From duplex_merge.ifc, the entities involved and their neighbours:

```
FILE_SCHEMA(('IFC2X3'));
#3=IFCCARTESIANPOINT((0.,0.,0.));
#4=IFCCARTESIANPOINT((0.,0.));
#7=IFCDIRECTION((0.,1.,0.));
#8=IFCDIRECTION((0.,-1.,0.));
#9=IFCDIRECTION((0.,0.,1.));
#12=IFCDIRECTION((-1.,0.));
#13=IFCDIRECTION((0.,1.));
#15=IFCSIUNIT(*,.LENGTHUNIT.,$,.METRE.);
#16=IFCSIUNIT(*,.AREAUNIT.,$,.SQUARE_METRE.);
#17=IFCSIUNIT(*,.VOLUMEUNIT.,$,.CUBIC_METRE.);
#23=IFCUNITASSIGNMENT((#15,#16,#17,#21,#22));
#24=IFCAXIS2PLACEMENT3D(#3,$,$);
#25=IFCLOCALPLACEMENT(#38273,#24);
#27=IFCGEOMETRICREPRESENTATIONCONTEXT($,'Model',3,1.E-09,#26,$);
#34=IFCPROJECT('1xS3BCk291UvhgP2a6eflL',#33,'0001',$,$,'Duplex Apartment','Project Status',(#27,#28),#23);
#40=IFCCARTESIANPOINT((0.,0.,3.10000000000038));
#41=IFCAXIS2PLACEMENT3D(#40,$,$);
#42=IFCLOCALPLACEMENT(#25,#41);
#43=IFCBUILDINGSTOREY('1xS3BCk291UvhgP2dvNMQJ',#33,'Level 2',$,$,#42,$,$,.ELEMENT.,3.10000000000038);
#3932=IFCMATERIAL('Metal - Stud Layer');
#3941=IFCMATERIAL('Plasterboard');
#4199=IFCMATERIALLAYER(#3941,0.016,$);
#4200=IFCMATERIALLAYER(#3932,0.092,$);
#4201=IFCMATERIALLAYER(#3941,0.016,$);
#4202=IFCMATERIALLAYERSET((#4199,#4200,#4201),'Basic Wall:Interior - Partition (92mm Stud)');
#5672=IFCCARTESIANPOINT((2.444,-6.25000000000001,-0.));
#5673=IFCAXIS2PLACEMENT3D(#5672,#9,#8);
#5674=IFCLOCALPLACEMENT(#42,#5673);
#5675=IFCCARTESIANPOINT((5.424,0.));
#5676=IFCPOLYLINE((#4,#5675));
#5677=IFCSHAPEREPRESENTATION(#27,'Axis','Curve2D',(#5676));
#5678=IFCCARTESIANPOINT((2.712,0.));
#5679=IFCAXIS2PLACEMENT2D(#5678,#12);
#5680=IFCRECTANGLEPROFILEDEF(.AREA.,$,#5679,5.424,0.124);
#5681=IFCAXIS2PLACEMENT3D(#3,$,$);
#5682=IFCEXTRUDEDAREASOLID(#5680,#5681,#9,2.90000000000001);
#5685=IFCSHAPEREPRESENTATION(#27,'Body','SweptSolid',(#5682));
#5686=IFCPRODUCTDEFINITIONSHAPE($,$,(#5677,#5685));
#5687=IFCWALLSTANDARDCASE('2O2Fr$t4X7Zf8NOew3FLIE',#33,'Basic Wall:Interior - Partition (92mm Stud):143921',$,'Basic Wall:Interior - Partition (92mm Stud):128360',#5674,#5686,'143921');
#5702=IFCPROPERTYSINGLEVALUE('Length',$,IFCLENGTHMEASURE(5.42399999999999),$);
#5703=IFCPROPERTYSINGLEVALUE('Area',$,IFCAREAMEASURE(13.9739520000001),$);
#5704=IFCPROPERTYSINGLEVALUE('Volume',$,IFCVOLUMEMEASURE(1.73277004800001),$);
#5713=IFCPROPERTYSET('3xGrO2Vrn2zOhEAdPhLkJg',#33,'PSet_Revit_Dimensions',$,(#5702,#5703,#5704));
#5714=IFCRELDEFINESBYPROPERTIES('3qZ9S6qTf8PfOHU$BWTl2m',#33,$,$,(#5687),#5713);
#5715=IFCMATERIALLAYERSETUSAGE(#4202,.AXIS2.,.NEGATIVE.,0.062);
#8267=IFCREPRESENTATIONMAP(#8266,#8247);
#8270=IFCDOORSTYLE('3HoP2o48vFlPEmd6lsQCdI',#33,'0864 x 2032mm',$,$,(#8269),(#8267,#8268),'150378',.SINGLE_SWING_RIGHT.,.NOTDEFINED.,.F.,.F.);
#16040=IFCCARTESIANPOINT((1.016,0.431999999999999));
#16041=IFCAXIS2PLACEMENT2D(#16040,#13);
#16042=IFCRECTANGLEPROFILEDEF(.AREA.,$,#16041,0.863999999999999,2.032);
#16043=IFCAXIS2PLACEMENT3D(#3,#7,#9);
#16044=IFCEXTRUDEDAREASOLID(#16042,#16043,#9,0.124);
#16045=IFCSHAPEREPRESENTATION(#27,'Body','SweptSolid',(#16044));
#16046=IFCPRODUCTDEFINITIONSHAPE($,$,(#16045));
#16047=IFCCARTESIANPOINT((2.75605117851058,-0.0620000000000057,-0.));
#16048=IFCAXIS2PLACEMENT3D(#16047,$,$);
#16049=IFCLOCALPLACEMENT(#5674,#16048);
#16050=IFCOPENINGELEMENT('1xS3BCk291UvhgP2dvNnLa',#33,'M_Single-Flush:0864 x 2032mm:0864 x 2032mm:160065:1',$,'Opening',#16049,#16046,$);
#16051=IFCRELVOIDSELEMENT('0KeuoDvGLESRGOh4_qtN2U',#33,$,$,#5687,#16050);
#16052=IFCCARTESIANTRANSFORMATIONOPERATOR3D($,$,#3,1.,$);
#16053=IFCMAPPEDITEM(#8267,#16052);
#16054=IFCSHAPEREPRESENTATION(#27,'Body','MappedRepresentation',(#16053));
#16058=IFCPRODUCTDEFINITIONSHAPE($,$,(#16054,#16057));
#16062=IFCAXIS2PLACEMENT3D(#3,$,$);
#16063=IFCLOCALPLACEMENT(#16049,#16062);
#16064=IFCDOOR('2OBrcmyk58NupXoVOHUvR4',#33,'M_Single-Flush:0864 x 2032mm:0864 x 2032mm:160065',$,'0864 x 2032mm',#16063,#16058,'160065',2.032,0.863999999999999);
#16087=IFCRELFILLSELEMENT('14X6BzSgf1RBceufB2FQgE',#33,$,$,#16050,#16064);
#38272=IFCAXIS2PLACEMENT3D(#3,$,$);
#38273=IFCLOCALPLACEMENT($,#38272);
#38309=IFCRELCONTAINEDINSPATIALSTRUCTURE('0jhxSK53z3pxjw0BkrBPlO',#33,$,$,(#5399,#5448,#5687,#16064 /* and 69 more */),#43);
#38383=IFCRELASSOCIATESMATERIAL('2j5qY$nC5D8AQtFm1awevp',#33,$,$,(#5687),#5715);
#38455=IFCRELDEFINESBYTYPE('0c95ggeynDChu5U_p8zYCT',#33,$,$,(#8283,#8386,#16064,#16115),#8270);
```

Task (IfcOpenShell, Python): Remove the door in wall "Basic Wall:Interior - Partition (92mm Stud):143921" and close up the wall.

```python
import ifcopenshell
import ifcopenshell.api.feature
import ifcopenshell.api.pset
import ifcopenshell.api.root
import ifcopenshell.geom
import ifcopenshell.util.element
import ifcopenshell.util.shape
import ifcopenshell.util.unit

model = ifcopenshell.open("duplex_merge.ifc")
area_scale = ifcopenshell.util.unit.calculate_unit_scale(model, "AREAUNIT")
volume_scale = ifcopenshell.util.unit.calculate_unit_scale(model, "VOLUMEUNIT")
settings = ifcopenshell.geom.settings()


def volume(element):
    """Net volume in cubic metres, openings subtracted."""
    shape = ifcopenshell.geom.create_shape(settings, element)
    return ifcopenshell.util.shape.get_volume(shape.geometry)


door = model.by_guid("2OBrcmyk58NupXoVOHUvR4")
opening = door.FillsVoids[0].RelatingOpeningElement
wall = opening.VoidsElements[0].RelatingBuildingElement
before = volume(wall)

ifcopenshell.api.root.remove_product(model, product=door)
ifcopenshell.api.feature.remove_feature(model, feature=opening)

after = volume(wall)
thickness = 0.124  # wall thickness in metres

# Update the wall's stored quantities.
pset = model.by_id(ifcopenshell.util.element.get_pset(wall, "PSet_Revit_Dimensions", should_inherit=False)["id"])
ifcopenshell.api.pset.edit_pset(model, pset=pset, properties={
    "Area": model.create_entity("IfcAreaMeasure", after / thickness / area_scale),
    "Volume": model.create_entity("IfcVolumeMeasure", after / volume_scale),
})

print(f"wall volume {before:.3f} -> {after:.3f} m3")

model.write("duplex_merge_rev.ifc")
```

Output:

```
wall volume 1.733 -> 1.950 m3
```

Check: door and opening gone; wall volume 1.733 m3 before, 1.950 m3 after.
